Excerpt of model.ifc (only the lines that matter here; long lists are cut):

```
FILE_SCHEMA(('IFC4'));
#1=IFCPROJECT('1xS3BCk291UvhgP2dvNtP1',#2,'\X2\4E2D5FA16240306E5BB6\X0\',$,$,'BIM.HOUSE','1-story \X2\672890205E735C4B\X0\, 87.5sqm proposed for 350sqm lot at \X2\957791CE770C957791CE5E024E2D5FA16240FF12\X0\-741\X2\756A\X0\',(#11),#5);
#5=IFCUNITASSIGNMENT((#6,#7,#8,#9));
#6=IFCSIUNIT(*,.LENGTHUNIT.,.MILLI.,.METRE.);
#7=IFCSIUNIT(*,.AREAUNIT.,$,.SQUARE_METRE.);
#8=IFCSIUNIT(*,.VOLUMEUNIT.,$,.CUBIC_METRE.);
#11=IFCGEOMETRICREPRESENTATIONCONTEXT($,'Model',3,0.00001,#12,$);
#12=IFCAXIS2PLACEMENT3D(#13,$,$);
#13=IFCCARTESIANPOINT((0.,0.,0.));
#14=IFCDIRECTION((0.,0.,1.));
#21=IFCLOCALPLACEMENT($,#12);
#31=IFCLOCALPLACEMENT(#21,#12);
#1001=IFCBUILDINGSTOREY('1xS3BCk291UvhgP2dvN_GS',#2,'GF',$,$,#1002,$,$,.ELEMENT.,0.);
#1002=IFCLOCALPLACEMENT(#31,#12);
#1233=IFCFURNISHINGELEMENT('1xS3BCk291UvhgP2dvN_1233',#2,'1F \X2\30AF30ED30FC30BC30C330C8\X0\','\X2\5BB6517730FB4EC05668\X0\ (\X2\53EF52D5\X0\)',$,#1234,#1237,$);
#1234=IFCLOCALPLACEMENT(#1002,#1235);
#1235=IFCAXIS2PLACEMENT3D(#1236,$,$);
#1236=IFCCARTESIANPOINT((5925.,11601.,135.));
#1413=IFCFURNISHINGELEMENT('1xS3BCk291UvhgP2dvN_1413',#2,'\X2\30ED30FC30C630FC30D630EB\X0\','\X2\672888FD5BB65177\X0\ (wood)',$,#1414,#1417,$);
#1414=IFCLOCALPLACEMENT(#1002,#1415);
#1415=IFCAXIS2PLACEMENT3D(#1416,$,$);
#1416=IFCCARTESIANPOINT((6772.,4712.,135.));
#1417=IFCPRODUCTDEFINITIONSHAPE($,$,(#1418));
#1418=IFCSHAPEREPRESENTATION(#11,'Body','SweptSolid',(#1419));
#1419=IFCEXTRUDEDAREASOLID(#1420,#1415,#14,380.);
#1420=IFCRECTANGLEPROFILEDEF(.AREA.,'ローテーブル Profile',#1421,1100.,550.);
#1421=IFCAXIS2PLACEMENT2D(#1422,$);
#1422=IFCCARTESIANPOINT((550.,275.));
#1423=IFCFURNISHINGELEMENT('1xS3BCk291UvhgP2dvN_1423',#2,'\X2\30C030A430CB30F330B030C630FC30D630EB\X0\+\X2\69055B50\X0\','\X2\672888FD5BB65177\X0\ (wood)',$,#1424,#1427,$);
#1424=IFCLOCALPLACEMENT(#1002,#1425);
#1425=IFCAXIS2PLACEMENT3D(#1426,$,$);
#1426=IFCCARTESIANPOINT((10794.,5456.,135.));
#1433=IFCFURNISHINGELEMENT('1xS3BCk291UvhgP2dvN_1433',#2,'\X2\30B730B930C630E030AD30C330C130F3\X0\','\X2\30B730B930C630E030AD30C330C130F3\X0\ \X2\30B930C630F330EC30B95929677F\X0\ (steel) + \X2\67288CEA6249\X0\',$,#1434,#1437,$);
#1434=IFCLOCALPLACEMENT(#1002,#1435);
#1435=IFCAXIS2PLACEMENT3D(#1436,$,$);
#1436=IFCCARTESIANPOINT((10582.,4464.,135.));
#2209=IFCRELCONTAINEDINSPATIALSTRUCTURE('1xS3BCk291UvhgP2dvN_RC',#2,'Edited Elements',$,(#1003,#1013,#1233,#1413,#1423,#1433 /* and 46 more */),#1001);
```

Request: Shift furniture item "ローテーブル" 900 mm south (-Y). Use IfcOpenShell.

```python
import ifcopenshell
import ifcopenshell.api.geometry
import ifcopenshell.util.placement
import ifcopenshell.util.unit

model = ifcopenshell.open("model.ifc")
unit_scale = ifcopenshell.util.unit.calculate_unit_scale(model)

item = model.by_guid("1xS3BCk291UvhgP2dvN_1413")
matrix = ifcopenshell.util.placement.get_local_placement(item.ObjectPlacement)
matrix[1, 3] -= 0.9 / unit_scale
ifcopenshell.api.geometry.edit_object_placement(model, product=item, matrix=matrix, is_si=False)

print(ifcopenshell.util.placement.get_local_placement(item.ObjectPlacement).round(3) + 0.0)

model.write("model_v2.ifc")
```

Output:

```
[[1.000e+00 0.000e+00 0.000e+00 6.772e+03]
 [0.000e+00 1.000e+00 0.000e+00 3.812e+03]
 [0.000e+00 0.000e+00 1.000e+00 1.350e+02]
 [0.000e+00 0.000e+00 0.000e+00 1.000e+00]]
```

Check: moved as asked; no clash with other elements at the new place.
